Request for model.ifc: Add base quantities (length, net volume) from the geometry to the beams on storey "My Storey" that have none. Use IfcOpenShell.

First a look at what the model holds.

```python
import ifcopenshell
import ifcopenshell.util.element
import ifcopenshell.util.unit

model = ifcopenshell.open("model.ifc")
print(model.schema)
for unit_type in ("LENGTHUNIT", "AREAUNIT", "VOLUMEUNIT"):
    print(unit_type, ifcopenshell.util.unit.calculate_unit_scale(model, unit_type))
storey = next(s for s in model.by_type("IfcBuildingStorey") if s.Name == "My Storey")
beams = [e for e in ifcopenshell.util.element.get_decomposition(storey) if e.is_a("IfcBeam")]
for e in sorted(beams, key=lambda e: e.id()):
    print(e.id(), e.is_a(), e.Name, list(ifcopenshell.util.element.get_psets(e, qtos_only=True)), sep=" | ")
```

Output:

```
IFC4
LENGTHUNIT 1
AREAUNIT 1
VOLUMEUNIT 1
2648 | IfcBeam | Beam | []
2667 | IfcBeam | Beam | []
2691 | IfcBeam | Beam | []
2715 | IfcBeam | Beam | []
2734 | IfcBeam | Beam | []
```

```python
import ifcopenshell
import ifcopenshell.api.pset
import ifcopenshell.geom
import ifcopenshell.util.element
import ifcopenshell.util.shape
import ifcopenshell.util.unit

model = ifcopenshell.open("model.ifc")
unit_scale = ifcopenshell.util.unit.calculate_unit_scale(model)
volume_scale = ifcopenshell.util.unit.calculate_unit_scale(model, "VOLUMEUNIT")
settings = ifcopenshell.geom.settings()

storey = next(s for s in model.by_type("IfcBuildingStorey") if s.Name == "My Storey")
beams = [e for e in ifcopenshell.util.element.get_decomposition(storey) if e.is_a("IfcBeam")]

for e in sorted(beams, key=lambda e: e.id()):
    if ifcopenshell.util.element.get_psets(e, qtos_only=True, should_inherit=False):
        continue
    # Geometry comes back in metres, in the element's own axes.
    shape = ifcopenshell.geom.create_shape(settings, e)
    values = {
        "Length": ifcopenshell.util.shape.get_max_xyz(shape.geometry) / unit_scale,
        "NetVolume": ifcopenshell.util.shape.get_volume(shape.geometry) / volume_scale,
    }
    qto = ifcopenshell.api.pset.add_qto(model, product=e, name="Qto_BeamBaseQuantities")
    ifcopenshell.api.pset.edit_qto(model, qto=qto, properties=values)
    print(e.id(), {k: round(v, 3) for k, v in values.items()})

model.write("model_edited.ifc")
```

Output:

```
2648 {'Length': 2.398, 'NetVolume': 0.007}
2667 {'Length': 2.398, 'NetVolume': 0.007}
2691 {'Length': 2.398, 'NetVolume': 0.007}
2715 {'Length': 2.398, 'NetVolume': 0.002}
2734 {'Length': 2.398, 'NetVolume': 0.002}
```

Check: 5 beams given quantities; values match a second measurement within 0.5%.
